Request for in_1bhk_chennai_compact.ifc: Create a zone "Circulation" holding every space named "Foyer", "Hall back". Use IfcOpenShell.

First a look at what the model holds.

```python
import ifcopenshell

model = ifcopenshell.open("in_1bhk_chennai_compact.ifc")
print(model.schema)
seen = {}
for space in model.by_type("IfcSpace"):
    seen[space.LongName] = seen.get(space.LongName, 0) + 1
for name, count in sorted(seen.items(), key=str):
    print(count, "x", name)
print("zones:", [z.Name for z in model.by_type("IfcZone")][:20])
```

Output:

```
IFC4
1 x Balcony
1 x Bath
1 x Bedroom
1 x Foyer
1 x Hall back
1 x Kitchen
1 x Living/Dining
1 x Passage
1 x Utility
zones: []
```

```python
import ifcopenshell
import ifcopenshell.api.group
import ifcopenshell.api.root

model = ifcopenshell.open("in_1bhk_chennai_compact.ifc")

names = {"Foyer", "Hall back"}
spaces = [s for s in model.by_type("IfcSpace") if s.LongName in names]

zone = ifcopenshell.api.root.create_entity(model, ifc_class="IfcZone", name="Circulation")
ifcopenshell.api.group.assign_group(model, products=spaces, group=zone)
print(len(spaces), "spaces in", zone.Name)

model.write("in_1bhk_chennai_compact_updated.ifc")
```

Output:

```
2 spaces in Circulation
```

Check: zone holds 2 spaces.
